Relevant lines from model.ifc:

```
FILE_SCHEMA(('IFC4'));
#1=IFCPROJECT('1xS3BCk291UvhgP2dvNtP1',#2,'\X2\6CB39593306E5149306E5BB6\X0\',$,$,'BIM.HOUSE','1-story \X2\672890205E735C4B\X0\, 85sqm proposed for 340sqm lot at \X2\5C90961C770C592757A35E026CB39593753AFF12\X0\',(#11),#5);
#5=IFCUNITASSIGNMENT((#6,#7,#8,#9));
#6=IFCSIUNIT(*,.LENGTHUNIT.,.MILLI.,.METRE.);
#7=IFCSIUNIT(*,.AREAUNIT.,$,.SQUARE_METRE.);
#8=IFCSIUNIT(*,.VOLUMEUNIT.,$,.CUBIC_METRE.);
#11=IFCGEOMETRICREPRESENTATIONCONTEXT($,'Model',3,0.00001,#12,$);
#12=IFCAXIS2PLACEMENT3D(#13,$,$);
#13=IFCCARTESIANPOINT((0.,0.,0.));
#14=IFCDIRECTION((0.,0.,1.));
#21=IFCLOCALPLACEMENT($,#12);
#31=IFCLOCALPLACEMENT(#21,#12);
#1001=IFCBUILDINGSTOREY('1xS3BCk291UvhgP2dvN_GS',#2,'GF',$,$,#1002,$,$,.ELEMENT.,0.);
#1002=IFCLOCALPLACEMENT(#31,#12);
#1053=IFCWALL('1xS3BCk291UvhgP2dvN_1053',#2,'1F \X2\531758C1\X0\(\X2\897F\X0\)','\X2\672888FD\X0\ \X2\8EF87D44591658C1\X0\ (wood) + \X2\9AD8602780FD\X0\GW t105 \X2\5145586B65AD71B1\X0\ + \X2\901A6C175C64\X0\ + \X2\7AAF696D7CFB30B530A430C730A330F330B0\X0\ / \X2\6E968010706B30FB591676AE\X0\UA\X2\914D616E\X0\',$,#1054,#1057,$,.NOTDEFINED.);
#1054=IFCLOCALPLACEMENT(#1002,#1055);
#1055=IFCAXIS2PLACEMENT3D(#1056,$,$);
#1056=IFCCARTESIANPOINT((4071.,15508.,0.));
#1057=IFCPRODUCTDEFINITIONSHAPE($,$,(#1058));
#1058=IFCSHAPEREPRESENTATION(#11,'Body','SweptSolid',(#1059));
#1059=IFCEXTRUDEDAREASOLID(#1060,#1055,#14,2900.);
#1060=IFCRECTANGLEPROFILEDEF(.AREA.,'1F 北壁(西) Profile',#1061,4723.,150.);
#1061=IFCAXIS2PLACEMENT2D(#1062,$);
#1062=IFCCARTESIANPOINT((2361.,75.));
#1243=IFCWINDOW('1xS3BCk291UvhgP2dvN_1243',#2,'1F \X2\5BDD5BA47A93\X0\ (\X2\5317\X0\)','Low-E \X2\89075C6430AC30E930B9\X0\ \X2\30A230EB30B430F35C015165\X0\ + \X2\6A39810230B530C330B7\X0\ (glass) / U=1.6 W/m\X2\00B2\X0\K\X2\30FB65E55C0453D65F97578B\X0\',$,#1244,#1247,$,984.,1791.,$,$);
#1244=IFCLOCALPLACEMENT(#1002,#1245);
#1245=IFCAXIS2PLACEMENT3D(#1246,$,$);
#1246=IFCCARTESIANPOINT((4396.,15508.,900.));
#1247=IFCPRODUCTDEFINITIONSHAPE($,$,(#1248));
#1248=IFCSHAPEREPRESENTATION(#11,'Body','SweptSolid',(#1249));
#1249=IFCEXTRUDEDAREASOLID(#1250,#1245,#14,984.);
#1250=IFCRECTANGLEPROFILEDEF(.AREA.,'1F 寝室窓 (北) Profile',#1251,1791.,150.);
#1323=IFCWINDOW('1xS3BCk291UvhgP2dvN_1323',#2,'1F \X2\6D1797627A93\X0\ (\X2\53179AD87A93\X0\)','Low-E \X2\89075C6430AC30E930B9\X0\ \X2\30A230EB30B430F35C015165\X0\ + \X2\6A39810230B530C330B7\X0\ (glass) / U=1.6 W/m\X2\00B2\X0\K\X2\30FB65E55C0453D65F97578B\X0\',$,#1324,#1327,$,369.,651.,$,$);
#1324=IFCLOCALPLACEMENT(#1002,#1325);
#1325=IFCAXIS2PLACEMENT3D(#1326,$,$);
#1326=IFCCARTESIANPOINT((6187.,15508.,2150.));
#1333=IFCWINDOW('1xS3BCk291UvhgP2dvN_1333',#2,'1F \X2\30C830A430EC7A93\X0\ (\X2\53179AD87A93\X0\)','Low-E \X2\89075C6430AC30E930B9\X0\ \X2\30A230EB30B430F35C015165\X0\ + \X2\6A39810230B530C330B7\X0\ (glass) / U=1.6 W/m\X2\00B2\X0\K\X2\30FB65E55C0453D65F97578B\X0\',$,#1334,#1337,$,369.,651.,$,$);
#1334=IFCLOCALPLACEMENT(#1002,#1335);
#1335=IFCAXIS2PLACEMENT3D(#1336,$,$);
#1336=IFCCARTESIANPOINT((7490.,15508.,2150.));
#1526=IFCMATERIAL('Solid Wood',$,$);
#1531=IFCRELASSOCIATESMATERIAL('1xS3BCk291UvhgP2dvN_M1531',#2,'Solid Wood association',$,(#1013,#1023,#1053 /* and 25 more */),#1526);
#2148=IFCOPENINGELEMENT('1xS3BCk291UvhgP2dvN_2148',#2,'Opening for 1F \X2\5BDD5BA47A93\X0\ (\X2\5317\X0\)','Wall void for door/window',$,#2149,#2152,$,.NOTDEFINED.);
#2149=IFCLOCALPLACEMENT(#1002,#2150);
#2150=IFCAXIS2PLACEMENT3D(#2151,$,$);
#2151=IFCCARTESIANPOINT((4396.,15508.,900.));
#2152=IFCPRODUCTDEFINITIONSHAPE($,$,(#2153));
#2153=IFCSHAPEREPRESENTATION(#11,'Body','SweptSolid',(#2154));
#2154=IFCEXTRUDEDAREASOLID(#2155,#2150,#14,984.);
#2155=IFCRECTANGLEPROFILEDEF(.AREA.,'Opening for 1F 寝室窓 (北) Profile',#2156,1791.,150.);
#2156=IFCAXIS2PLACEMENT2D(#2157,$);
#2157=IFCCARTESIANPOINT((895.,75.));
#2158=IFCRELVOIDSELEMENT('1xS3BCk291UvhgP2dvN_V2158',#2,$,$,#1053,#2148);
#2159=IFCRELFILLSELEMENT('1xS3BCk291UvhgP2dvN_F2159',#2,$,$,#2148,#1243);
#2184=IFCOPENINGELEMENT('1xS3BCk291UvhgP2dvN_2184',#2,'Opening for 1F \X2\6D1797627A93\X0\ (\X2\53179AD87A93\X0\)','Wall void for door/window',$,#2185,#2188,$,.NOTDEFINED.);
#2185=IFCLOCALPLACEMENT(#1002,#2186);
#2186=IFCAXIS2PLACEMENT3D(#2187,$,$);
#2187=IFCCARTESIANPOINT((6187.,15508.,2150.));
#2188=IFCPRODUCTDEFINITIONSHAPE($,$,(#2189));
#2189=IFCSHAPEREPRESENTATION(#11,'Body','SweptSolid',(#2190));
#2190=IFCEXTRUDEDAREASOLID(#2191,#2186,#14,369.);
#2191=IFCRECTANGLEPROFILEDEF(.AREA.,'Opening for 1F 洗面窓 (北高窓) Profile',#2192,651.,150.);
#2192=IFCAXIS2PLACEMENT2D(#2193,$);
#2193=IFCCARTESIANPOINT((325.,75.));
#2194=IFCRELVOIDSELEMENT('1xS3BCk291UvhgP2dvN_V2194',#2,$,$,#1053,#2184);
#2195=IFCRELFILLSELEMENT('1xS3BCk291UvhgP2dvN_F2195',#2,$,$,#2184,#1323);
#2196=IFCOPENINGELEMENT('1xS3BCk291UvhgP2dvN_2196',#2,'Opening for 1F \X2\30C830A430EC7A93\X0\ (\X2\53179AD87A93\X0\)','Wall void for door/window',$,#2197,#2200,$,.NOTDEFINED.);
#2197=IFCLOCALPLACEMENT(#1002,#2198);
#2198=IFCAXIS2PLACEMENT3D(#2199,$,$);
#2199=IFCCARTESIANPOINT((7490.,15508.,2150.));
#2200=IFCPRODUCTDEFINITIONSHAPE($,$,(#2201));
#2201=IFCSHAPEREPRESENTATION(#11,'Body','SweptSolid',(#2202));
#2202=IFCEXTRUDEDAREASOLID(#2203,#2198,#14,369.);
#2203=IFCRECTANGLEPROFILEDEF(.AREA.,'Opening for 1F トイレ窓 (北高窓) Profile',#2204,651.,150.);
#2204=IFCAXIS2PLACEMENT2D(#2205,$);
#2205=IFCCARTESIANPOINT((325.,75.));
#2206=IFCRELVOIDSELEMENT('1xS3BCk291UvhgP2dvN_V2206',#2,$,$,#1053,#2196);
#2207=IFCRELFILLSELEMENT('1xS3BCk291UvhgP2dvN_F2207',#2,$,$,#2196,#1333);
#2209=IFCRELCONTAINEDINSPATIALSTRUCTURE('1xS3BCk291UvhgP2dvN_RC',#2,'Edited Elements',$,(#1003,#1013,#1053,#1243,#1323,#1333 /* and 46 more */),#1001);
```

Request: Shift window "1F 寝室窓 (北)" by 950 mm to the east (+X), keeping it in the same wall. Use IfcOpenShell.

```python
import ifcopenshell
import ifcopenshell.api.geometry
import ifcopenshell.util.placement

model = ifcopenshell.open("model.ifc")

window = model.by_guid("1xS3BCk291UvhgP2dvN_1243")
opening = window.FillsVoids[0].RelatingOpeningElement
wall = opening.VoidsElements[0].RelatingBuildingElement

wall_matrix = ifcopenshell.util.placement.get_local_placement(wall.ObjectPlacement)
shift = wall_matrix[:3, 0] * 950.0
before = ifcopenshell.util.placement.get_local_placement(window.ObjectPlacement)[:3, 3].copy()

# The window is not placed relative to its opening, so move both.
for product in (opening, window):
    matrix = ifcopenshell.util.placement.get_local_placement(product.ObjectPlacement)
    matrix[:3, 3] += shift
    ifcopenshell.api.geometry.edit_object_placement(model, product=product, matrix=matrix, is_si=False)

after = ifcopenshell.util.placement.get_local_placement(window.ObjectPlacement)[:3, 3]
print("window moved by", (after - before).round(3) + 0.0)

model.write("model_updated.ifc")
```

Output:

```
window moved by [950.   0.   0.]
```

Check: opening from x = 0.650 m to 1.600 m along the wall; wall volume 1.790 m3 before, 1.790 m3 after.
